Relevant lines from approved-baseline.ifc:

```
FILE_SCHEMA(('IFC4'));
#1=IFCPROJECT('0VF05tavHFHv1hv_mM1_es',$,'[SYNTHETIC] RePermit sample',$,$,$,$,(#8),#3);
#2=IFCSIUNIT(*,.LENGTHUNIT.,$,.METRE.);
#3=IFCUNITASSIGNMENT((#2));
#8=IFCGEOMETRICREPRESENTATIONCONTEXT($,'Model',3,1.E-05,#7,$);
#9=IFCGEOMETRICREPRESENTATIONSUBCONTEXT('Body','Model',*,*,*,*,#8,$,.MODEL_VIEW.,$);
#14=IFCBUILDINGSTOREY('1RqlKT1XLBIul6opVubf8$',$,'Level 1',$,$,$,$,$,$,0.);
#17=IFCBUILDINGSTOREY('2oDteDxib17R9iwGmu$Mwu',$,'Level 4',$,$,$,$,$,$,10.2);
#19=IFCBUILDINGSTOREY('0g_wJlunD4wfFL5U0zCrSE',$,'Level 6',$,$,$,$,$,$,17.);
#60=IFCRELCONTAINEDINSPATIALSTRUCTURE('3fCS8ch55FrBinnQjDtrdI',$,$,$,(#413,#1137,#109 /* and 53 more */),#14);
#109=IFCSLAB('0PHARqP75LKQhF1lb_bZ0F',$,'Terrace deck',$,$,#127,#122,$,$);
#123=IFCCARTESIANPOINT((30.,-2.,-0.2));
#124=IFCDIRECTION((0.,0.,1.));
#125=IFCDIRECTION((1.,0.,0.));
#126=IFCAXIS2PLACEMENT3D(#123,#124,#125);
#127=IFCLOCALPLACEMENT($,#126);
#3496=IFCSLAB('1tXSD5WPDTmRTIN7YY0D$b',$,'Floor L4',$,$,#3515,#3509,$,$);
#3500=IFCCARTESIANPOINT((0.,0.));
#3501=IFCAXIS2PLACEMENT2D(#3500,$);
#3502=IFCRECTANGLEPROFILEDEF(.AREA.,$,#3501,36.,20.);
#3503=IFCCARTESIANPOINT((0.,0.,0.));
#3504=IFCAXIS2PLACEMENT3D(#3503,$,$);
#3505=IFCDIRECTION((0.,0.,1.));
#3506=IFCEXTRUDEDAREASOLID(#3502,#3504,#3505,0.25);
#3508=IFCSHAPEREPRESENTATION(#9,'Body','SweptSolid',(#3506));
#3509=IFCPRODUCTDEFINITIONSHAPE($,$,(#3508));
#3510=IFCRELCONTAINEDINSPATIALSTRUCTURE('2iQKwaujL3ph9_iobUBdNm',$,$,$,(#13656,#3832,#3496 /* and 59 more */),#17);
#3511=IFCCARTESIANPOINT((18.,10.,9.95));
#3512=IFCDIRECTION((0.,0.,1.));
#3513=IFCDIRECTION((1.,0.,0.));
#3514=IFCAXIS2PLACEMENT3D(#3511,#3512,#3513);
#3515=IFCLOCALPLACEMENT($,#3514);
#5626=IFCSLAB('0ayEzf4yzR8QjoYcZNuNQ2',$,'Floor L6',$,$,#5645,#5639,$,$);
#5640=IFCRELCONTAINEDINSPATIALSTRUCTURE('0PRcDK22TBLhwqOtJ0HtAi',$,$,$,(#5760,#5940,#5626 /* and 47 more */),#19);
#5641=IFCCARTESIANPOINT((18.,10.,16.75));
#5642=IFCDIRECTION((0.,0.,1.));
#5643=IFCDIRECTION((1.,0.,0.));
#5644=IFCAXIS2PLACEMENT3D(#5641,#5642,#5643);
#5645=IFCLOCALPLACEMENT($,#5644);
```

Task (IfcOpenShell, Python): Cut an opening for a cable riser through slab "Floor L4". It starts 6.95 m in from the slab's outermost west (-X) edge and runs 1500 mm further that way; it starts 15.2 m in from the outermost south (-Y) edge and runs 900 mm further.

```python
import numpy as np
import ifcopenshell
import ifcopenshell.api.feature
import ifcopenshell.api.geometry
import ifcopenshell.api.root
import ifcopenshell.geom
import ifcopenshell.util.placement
import ifcopenshell.util.representation
import ifcopenshell.util.shape
import ifcopenshell.util.unit

model = ifcopenshell.open("approved-baseline.ifc")
unit_scale = ifcopenshell.util.unit.calculate_unit_scale(model)
settings = ifcopenshell.geom.settings()


def volume(element):
    """Net volume in cubic metres, openings subtracted."""
    shape = ifcopenshell.geom.create_shape(settings, element)
    return ifcopenshell.util.shape.get_volume(shape.geometry)


slab = model.by_guid("1tXSD5WPDTmRTIN7YY0D$b")
before = volume(slab)

# Extent in the slab's own axes, in metres. The edges named are its -X and -Y sides.
slab_shape = ifcopenshell.geom.create_shape(settings, slab)
vertices = ifcopenshell.util.shape.get_vertices(slab_shape.geometry)
x_min, y_min, bottom = vertices.min(axis=0)
top = vertices[:, 2].max()

opening = ifcopenshell.api.root.create_entity(model, ifc_class="IfcOpeningElement", name="Cable riser opening", predefined_type="OPENING")
context = ifcopenshell.util.representation.get_context(model, "Model", "Body", "MODEL_VIEW")
width, depth = 1.5, 0.9
outline = [(0.0, 0.0), (width, 0.0), (width, depth), (0.0, depth), (0.0, 0.0)]
# Overshoot both faces by 50 mm so the cut is clean.
shape = ifcopenshell.api.geometry.add_slab_representation(
    model, context=context, depth=top - bottom + 0.1, polyline=outline
)
ifcopenshell.api.geometry.assign_representation(model, product=opening, representation=shape)

matrix = ifcopenshell.util.placement.get_local_placement(slab.ObjectPlacement)
matrix[:, 3] = matrix @ np.append(np.array([x_min + 6.95, y_min + 15.2, bottom - 0.05]) / unit_scale, 1.0)
ifcopenshell.api.geometry.edit_object_placement(model, product=opening, matrix=matrix, is_si=False)
ifcopenshell.api.feature.add_feature(model, feature=opening, element=slab)

after = volume(slab)

print(f"slab volume {before:.3f} -> {after:.3f} m3")

model.write("approved-baseline_rev.ifc")
```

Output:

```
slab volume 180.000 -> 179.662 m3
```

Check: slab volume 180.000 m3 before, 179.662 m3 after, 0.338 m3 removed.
